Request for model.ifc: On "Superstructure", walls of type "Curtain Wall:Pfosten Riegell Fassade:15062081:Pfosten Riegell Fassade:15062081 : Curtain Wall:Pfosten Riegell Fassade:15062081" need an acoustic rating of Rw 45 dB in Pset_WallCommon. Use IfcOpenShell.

First a look at what the model holds.

```python
import ifcopenshell
import ifcopenshell.util.element

model = ifcopenshell.open("model.ifc")
print(model.schema)
storey = next(s for s in model.by_type("IfcBuildingStorey") if s.Name == "Superstructure")
walls = [e for e in ifcopenshell.util.element.get_decomposition(storey) if e.is_a("IfcWall")]
seen = {}
for e in walls:
    element_type = ifcopenshell.util.element.get_type(e)
    key = (element_type.Name if element_type != e and element_type else None, ifcopenshell.util.element.get_pset(e, "Pset_WallCommon", "AcousticRating"))
    seen[key] = seen.get(key, 0) + 1
for (name, value), count in sorted(seen.items(), key=str):
    print(count, "x", name, "|", value)
```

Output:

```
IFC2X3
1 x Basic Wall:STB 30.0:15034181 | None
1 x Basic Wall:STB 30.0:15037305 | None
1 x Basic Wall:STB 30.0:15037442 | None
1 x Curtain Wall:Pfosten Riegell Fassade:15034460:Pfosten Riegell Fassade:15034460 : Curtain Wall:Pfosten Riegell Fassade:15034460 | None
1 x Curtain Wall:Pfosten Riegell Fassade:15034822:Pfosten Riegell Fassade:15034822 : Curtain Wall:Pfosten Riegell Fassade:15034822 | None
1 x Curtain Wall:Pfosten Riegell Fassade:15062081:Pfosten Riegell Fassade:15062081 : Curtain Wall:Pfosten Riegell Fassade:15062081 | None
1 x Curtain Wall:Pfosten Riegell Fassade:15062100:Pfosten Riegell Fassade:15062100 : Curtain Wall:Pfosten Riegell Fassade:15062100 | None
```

```python
import ifcopenshell
import ifcopenshell.api.pset
import ifcopenshell.util.element

model = ifcopenshell.open("model.ifc")

storey = next(s for s in model.by_type("IfcBuildingStorey") if s.Name == "Superstructure")
walls = [e for e in ifcopenshell.util.element.get_decomposition(storey) if e.is_a("IfcWall")]

count = 0
for e in walls:
    element_type = ifcopenshell.util.element.get_type(e)
    if element_type in (None, e) or element_type.Name != "Curtain Wall:Pfosten Riegell Fassade:15062081:Pfosten Riegell Fassade:15062081 : Curtain Wall:Pfosten Riegell Fassade:15062081":
        continue
    # add_pset returns the element's existing set when there is one.
    pset = ifcopenshell.api.pset.add_pset(model, product=e, name="Pset_WallCommon")
    ifcopenshell.api.pset.edit_pset(model, pset=pset, properties={"AcousticRating": "Rw 45 dB"})
    count += 1

print(count, "walls updated")

model.write("model_rev.ifc")
```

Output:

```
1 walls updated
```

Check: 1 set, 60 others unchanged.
